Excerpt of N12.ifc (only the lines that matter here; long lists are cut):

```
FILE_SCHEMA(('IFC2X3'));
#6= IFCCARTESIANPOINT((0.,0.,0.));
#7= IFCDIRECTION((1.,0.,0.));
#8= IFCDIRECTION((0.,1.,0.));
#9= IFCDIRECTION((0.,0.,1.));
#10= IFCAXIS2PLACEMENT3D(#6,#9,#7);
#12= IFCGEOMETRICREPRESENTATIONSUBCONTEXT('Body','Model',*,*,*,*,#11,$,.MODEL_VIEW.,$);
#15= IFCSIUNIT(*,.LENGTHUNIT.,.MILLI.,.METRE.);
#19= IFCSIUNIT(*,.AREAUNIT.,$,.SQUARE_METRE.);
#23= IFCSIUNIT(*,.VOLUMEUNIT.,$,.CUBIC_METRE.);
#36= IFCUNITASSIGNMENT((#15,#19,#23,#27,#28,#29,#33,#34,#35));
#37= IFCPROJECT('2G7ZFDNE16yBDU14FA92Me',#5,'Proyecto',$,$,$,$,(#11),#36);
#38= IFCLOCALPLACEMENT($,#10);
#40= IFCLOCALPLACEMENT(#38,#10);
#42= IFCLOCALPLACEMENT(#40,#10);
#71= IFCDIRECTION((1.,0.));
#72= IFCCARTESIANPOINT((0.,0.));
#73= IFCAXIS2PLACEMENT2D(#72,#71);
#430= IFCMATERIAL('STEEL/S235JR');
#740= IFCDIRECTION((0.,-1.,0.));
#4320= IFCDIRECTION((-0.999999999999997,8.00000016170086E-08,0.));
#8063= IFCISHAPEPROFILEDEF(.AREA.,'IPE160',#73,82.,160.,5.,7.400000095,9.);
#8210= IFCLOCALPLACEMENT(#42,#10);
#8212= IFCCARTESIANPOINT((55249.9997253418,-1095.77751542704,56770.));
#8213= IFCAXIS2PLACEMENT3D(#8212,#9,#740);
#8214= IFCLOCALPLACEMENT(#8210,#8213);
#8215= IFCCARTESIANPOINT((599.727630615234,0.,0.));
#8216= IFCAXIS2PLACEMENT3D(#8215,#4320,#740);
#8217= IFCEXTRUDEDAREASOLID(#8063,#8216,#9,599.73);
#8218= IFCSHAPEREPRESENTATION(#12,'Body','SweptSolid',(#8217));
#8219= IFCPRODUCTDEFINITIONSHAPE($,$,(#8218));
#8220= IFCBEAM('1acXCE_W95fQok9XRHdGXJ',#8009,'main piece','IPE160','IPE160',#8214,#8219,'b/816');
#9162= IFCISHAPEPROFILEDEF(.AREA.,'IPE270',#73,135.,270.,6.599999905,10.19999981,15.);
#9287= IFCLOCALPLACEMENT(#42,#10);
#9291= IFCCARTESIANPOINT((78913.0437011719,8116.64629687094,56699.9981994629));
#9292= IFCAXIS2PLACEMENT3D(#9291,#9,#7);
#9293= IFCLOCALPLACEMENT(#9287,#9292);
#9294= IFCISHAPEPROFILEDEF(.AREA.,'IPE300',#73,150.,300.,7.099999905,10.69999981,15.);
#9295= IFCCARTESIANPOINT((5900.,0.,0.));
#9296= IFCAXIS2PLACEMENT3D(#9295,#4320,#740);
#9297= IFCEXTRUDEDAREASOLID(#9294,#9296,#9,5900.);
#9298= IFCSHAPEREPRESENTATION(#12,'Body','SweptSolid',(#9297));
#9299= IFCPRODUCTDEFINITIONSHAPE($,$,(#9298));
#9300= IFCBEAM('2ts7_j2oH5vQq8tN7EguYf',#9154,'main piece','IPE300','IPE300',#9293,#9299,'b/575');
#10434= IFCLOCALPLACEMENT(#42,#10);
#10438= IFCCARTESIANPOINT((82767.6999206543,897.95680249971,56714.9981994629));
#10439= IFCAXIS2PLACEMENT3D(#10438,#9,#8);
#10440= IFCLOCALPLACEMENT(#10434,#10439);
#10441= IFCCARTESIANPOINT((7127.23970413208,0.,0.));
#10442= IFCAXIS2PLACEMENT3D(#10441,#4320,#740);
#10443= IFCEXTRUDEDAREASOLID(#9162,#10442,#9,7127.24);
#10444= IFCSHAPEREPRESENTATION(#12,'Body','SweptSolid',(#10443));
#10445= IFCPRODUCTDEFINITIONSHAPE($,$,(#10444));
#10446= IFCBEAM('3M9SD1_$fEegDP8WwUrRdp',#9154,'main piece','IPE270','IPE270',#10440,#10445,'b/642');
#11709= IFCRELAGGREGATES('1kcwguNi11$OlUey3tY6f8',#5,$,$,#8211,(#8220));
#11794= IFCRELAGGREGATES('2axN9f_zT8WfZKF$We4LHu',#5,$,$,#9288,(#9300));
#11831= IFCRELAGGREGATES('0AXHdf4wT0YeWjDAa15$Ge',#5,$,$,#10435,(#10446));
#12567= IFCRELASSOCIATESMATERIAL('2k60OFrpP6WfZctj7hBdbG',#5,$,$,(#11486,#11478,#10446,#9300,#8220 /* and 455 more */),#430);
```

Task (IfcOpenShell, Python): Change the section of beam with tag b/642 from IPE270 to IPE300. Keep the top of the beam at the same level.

```python
import ifcopenshell
import ifcopenshell.util.element
import ifcopenshell.util.representation

model = ifcopenshell.open("N12.ifc")

member = model.by_id(10446)
source = next(p for p in model.by_type("IfcIShapeProfileDef") if p.ProfileName == "IPE300")

body = ifcopenshell.util.representation.get_representation(member, "Model", "Body")
solid = body.Items[0]
old_profile = solid.SweptArea

# Copy the section's sizes but keep this member's own profile position.
profile = ifcopenshell.util.element.copy(model, source)
# Profiles are centred, so shift by half the change in depth to hold the top.
shift = (old_profile.OverallDepth - profile.OverallDepth) / 2
x, y = old_profile.Position.Location.Coordinates
up = (0.0, 1.0)  # upwards, in the solid's own plane
location = model.createIfcCartesianPoint((x + up[0] * shift, y + up[1] * shift))
profile.Position = model.createIfcAxis2Placement2D(location, old_profile.Position.RefDirection)
solid.SweptArea = profile
if not model.get_total_inverses(old_profile):
    ifcopenshell.util.element.remove_deep2(model, old_profile)
member.Description = member.Description.replace("IPE270", "IPE300")
member.ObjectType = member.ObjectType.replace("IPE270", "IPE300")

print(solid.SweptArea)

model.write("N12_updated.ifc")
```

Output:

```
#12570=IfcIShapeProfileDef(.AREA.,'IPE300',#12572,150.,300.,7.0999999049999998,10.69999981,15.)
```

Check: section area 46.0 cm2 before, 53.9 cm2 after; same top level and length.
